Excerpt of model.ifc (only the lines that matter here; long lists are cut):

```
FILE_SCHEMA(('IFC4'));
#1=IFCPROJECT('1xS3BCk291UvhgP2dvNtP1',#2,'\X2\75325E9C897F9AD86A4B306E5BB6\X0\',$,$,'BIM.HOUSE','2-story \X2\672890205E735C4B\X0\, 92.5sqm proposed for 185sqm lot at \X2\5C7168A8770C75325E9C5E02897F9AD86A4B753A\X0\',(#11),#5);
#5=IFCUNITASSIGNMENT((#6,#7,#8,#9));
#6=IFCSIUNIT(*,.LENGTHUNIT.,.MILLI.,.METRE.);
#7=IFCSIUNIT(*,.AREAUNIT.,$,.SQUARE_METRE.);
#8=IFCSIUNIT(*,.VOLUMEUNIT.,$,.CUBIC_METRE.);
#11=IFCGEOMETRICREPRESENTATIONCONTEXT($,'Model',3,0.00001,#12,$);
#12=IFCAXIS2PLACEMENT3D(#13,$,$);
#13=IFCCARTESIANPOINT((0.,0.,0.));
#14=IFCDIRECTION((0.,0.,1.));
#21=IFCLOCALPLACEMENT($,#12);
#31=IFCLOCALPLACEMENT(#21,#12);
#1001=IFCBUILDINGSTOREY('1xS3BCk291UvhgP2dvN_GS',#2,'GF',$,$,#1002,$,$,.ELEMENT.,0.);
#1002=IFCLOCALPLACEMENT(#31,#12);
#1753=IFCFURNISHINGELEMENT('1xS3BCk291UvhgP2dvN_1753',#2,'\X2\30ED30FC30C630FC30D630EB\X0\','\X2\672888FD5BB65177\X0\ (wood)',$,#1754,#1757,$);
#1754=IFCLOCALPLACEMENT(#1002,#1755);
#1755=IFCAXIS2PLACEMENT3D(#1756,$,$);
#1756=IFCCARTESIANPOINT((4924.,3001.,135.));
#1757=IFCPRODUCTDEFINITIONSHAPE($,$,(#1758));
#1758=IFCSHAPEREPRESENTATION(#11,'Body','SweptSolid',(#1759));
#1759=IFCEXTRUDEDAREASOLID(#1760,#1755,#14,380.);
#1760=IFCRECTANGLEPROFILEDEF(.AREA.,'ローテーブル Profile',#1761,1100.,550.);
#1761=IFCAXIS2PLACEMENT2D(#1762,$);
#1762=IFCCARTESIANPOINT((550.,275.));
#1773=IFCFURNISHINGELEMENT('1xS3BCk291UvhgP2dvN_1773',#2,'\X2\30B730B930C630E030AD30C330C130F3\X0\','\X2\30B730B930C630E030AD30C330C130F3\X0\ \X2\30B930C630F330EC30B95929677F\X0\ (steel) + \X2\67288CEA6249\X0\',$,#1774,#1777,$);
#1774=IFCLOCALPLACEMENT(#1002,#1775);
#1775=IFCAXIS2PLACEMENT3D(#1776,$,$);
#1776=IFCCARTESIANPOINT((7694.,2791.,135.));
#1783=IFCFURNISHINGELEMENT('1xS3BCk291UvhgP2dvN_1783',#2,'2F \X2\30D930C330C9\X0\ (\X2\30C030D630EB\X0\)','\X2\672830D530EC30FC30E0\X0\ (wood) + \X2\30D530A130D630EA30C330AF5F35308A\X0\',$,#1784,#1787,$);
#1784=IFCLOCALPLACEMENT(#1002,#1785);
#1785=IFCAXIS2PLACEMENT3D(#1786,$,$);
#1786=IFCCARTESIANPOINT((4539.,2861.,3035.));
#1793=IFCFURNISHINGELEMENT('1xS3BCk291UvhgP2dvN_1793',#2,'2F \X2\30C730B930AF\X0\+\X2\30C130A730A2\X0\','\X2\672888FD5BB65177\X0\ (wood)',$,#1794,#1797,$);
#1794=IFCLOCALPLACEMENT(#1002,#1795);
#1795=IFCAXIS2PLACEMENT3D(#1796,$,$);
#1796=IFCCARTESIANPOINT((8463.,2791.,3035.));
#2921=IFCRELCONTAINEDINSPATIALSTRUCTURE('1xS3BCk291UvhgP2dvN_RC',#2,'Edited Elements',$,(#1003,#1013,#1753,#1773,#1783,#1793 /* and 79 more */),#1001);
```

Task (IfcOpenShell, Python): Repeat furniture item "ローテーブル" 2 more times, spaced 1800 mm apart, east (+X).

```python
import numpy as np
import ifcopenshell
import ifcopenshell.api.geometry
import ifcopenshell.api.root
import ifcopenshell.util.element
import ifcopenshell.util.placement

model = ifcopenshell.open("model.ifc")


def reuse_history(source, copy):
    """copy_class also copies each property set's owner history, people and application; keep the originals."""
    for rel in copy.IsDefinedBy:
        if rel.is_a("IfcRelDefinesByProperties") and (history := rel.RelatingPropertyDefinition.OwnerHistory):
            rel.RelatingPropertyDefinition.OwnerHistory = source.OwnerHistory
            ifcopenshell.util.element.remove_deep2(model, history)


source = model.by_id(1753)
base = ifcopenshell.util.placement.get_local_placement(source.ObjectPlacement)
step = np.array([1.0, 0.0, 0.0]) * 1800.0

for i in range(1, 3):
    copy = ifcopenshell.api.root.copy_class(model, product=source)
    copy.Representation = ifcopenshell.util.element.copy_deep(
        model, source.Representation, exclude=["IfcGeometricRepresentationContext", "IfcRepresentationMap"]
    )
    reuse_history(source, copy)
    matrix = base.copy()
    matrix[:3, 3] += i * step
    print("added at", matrix[:3, 3].round(3) + 0.0)
    ifcopenshell.api.geometry.edit_object_placement(model, product=copy, matrix=matrix, is_si=False)

model.write("model_rev.ifc")
```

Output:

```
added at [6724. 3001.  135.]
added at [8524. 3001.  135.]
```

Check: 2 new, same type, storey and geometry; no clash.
